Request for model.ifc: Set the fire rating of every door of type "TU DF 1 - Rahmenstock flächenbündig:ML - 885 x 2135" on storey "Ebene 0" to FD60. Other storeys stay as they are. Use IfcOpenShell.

First a look at what the model holds.

```python
import ifcopenshell
import ifcopenshell.util.element

model = ifcopenshell.open("model.ifc")
print(model.schema)
storey = next(s for s in model.by_type("IfcBuildingStorey") if s.Name == "Ebene 0")
doors = [e for e in ifcopenshell.util.element.get_decomposition(storey) if e.is_a("IfcDoor")]
seen = {}
for e in doors:
    element_type = ifcopenshell.util.element.get_type(e)
    key = (element_type.Name if element_type != e and element_type else None, ifcopenshell.util.element.get_pset(e, "Pset_DoorCommon", "FireRating"))
    seen[key] = seen.get(key, 0) + 1
for (name, value), count in sorted(seen.items(), key=str):
    print(count, "x", name, "|", value)
```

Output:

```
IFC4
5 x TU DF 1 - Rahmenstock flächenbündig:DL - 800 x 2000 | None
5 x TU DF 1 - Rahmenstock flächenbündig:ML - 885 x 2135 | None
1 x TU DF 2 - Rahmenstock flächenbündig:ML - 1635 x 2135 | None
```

```python
import ifcopenshell
import ifcopenshell.api.pset
import ifcopenshell.util.element

model = ifcopenshell.open("model.ifc")

storey = next(s for s in model.by_type("IfcBuildingStorey") if s.Name == "Ebene 0")
doors = [e for e in ifcopenshell.util.element.get_decomposition(storey) if e.is_a("IfcDoor")]

count = 0
for e in doors:
    element_type = ifcopenshell.util.element.get_type(e)
    if element_type in (None, e) or element_type.Name != "TU DF 1 - Rahmenstock flächenbündig:ML - 885 x 2135":
        continue
    # add_pset returns the element's existing set when there is one.
    pset = ifcopenshell.api.pset.add_pset(model, product=e, name="Pset_DoorCommon")
    ifcopenshell.api.pset.edit_pset(model, pset=pset, properties={"FireRating": "FD60"})
    count += 1

print(count, "doors updated")

model.write("model_v2.ifc")
```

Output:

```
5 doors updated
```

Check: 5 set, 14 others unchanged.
